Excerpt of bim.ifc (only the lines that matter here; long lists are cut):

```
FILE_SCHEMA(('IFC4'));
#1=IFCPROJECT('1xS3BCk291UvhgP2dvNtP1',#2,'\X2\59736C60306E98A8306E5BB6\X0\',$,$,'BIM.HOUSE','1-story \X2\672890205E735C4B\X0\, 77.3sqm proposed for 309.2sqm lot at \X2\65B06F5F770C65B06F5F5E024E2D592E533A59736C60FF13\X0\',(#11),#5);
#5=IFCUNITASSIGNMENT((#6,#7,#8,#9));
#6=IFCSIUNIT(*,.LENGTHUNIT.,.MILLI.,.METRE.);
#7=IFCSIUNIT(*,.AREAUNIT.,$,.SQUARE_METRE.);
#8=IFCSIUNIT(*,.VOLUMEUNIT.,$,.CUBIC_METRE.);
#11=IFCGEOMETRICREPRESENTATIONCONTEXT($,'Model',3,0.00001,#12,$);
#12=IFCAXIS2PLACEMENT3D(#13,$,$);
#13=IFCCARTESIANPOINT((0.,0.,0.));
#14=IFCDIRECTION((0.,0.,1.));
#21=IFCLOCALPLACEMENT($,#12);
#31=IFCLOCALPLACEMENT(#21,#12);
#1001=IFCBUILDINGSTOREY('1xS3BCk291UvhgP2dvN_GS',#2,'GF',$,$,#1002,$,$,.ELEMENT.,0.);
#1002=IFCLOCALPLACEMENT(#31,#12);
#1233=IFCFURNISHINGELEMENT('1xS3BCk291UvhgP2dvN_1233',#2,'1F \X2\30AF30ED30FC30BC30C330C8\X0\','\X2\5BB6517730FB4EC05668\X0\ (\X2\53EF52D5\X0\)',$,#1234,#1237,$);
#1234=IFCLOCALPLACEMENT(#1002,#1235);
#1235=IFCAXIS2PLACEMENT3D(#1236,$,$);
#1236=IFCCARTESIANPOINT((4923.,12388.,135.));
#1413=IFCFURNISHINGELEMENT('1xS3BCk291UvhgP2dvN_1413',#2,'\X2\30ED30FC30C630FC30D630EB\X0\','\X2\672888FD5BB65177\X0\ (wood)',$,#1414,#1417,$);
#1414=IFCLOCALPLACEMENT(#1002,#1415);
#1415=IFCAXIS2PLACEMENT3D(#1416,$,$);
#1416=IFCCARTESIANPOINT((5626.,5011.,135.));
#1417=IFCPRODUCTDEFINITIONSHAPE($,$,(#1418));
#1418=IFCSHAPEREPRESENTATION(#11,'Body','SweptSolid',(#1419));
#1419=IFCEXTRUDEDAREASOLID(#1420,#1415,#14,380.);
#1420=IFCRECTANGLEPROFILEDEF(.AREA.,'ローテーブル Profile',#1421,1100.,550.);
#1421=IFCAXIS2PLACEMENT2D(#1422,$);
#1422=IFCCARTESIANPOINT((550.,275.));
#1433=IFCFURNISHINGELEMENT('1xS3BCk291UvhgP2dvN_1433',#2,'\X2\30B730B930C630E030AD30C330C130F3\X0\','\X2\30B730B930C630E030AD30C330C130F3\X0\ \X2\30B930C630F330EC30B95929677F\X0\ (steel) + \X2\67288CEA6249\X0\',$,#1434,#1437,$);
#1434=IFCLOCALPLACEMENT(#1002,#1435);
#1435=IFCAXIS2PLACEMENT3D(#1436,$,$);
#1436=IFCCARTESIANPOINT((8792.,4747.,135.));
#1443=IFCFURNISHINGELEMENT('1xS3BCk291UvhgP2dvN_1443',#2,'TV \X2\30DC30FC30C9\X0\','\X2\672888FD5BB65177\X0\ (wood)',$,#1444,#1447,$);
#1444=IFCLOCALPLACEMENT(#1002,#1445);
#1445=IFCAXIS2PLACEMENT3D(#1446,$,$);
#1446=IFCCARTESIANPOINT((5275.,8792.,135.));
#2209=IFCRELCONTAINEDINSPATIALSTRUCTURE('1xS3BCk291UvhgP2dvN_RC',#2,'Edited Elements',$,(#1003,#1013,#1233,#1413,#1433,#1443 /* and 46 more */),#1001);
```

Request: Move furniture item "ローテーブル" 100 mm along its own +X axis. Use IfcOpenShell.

```python
import ifcopenshell
import ifcopenshell.api.geometry
import ifcopenshell.util.placement

model = ifcopenshell.open("bim.ifc")

item = model.by_guid("1xS3BCk291UvhgP2dvN_1413")
matrix = ifcopenshell.util.placement.get_local_placement(item.ObjectPlacement)
matrix[:3, 3] += matrix[:3, 0] * 100.0
ifcopenshell.api.geometry.edit_object_placement(model, product=item, matrix=matrix, is_si=False)

print(ifcopenshell.util.placement.get_local_placement(item.ObjectPlacement).round(3) + 0.0)

model.write("bim_rev.ifc")
```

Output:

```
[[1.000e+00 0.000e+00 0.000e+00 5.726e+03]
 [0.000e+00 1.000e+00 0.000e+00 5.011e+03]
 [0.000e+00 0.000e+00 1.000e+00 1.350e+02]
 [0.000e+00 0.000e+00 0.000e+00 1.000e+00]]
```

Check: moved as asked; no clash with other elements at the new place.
